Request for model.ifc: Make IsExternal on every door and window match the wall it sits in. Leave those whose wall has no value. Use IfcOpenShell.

First a look at what the model holds.

```python
import ifcopenshell
import ifcopenshell.util.element

model = ifcopenshell.open("model.ifc")
print(model.schema)
seen = {}
for e in model.by_type("IfcDoor") + model.by_type("IfcWindow"):
    if not e.FillsVoids:
        continue
    host = e.FillsVoids[0].RelatingOpeningElement.VoidsElements[0].RelatingBuildingElement
    own = ifcopenshell.util.element.get_pset(e, f"Pset_{e.is_a()[3:].removesuffix('StandardCase')}Common", "IsExternal")
    wall = ifcopenshell.util.element.get_pset(host, "Pset_WallCommon", "IsExternal")
    seen[e.is_a(), own, wall] = seen.get((e.is_a(), own, wall), 0) + 1
for (cls, own, wall), count in sorted(seen.items(), key=str):
    print(count, cls, "IsExternal:", own, "| host wall:", wall)
```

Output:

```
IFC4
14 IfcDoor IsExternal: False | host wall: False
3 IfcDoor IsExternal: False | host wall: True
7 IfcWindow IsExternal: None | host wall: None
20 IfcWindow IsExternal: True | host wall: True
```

```python
import ifcopenshell
import ifcopenshell.api.pset
import ifcopenshell.util.element

model = ifcopenshell.open("model.ifc")

count = 0
for ifc_class, pset_name in (("IfcDoor", "Pset_DoorCommon"), ("IfcWindow", "Pset_WindowCommon")):
    for e in model.by_type(ifc_class):
        if not e.FillsVoids:
            continue
        host = e.FillsVoids[0].RelatingOpeningElement.VoidsElements[0].RelatingBuildingElement
        external = ifcopenshell.util.element.get_pset(host, "Pset_WallCommon", "IsExternal")
        if external is None or ifcopenshell.util.element.get_pset(e, pset_name, "IsExternal") == external:
            continue
        pset = ifcopenshell.api.pset.add_pset(model, product=e, name=pset_name)
        ifcopenshell.api.pset.edit_pset(model, pset=pset, properties={"IsExternal": external})
        count += 1

print(count, "updated")

model.write("model_updated.ifc")
```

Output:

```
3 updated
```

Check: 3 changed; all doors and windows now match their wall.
